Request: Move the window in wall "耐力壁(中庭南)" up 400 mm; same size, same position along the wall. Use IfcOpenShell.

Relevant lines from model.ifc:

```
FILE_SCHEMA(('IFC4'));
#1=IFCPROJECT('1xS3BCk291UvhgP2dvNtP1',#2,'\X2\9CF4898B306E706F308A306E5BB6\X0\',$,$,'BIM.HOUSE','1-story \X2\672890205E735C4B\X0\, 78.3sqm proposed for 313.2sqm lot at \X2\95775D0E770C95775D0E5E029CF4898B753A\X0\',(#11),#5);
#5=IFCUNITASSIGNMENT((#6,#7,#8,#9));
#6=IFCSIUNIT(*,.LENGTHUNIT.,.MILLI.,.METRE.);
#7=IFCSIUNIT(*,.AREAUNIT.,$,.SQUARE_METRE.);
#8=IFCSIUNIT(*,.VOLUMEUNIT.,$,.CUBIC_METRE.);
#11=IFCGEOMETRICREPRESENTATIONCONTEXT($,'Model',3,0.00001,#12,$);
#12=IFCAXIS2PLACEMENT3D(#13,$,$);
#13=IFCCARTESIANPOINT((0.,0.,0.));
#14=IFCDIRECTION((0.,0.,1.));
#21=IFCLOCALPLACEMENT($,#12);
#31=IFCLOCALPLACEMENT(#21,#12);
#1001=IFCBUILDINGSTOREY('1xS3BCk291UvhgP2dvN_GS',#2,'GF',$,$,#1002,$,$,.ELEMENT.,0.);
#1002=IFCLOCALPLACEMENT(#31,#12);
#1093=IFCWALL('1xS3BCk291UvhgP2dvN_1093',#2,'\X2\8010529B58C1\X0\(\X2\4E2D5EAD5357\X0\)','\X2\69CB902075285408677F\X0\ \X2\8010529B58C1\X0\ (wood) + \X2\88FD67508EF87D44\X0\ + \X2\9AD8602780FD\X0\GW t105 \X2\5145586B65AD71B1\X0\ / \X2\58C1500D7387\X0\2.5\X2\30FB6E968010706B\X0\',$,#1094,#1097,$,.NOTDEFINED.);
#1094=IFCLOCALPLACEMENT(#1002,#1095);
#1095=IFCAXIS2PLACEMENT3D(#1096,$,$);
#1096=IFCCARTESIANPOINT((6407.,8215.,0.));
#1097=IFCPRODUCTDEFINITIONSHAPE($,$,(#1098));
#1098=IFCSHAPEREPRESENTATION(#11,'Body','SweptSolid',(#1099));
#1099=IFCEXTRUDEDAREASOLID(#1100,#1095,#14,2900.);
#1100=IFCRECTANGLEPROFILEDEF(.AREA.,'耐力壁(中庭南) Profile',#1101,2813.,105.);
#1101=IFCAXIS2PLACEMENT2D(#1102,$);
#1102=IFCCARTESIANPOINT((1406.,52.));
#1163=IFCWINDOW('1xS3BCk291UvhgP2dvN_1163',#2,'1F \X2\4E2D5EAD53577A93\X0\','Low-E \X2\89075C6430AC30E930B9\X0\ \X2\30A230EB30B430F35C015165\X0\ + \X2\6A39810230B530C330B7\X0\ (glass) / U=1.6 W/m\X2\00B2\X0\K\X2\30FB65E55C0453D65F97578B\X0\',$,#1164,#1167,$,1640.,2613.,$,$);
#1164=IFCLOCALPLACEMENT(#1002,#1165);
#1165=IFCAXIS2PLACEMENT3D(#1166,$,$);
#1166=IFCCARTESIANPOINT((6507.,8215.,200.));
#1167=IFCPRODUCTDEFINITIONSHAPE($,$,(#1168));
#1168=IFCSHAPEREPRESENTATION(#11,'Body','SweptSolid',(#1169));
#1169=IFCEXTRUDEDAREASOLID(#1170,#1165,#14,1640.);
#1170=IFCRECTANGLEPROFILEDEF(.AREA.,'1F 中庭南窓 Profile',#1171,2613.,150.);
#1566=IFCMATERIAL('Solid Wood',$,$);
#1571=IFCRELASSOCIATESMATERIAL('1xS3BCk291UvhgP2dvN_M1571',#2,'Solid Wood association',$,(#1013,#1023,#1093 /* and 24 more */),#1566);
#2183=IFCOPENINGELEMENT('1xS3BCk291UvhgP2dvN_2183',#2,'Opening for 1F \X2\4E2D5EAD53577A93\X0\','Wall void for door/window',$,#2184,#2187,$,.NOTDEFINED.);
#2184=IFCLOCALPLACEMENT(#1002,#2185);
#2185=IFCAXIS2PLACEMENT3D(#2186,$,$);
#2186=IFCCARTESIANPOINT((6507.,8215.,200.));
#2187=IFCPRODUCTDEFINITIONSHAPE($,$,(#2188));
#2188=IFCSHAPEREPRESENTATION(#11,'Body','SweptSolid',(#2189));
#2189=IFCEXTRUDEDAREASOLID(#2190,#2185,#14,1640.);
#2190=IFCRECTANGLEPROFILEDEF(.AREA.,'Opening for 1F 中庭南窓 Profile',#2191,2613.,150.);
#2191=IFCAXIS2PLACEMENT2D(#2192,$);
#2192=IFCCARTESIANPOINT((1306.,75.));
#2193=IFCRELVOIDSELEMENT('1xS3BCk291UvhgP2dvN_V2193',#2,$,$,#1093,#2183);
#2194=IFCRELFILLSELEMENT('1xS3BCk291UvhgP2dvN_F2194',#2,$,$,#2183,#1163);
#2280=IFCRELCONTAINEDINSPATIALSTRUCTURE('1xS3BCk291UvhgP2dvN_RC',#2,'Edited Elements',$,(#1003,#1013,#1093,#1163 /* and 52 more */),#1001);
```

```python
import numpy as np
import ifcopenshell
import ifcopenshell.api.geometry
import ifcopenshell.util.placement
import ifcopenshell.util.unit

model = ifcopenshell.open("model.ifc")
unit_scale = ifcopenshell.util.unit.calculate_unit_scale(model)

window = model.by_id(1163)
opening = window.FillsVoids[0].RelatingOpeningElement
dz = 0.4 / unit_scale

shift = np.array([0.0, 0.0, dz])
# The window is not placed relative to its opening, so move both.
for product in (opening, window):
    matrix = ifcopenshell.util.placement.get_local_placement(product.ObjectPlacement)
    matrix[:3, 3] += shift
    ifcopenshell.api.geometry.edit_object_placement(model, product=product, matrix=matrix, is_si=False)

print(f"moved by {dz * unit_scale:+.3f} m")

model.write("model_rev.ifc")
```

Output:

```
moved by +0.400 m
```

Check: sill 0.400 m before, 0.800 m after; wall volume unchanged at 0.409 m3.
